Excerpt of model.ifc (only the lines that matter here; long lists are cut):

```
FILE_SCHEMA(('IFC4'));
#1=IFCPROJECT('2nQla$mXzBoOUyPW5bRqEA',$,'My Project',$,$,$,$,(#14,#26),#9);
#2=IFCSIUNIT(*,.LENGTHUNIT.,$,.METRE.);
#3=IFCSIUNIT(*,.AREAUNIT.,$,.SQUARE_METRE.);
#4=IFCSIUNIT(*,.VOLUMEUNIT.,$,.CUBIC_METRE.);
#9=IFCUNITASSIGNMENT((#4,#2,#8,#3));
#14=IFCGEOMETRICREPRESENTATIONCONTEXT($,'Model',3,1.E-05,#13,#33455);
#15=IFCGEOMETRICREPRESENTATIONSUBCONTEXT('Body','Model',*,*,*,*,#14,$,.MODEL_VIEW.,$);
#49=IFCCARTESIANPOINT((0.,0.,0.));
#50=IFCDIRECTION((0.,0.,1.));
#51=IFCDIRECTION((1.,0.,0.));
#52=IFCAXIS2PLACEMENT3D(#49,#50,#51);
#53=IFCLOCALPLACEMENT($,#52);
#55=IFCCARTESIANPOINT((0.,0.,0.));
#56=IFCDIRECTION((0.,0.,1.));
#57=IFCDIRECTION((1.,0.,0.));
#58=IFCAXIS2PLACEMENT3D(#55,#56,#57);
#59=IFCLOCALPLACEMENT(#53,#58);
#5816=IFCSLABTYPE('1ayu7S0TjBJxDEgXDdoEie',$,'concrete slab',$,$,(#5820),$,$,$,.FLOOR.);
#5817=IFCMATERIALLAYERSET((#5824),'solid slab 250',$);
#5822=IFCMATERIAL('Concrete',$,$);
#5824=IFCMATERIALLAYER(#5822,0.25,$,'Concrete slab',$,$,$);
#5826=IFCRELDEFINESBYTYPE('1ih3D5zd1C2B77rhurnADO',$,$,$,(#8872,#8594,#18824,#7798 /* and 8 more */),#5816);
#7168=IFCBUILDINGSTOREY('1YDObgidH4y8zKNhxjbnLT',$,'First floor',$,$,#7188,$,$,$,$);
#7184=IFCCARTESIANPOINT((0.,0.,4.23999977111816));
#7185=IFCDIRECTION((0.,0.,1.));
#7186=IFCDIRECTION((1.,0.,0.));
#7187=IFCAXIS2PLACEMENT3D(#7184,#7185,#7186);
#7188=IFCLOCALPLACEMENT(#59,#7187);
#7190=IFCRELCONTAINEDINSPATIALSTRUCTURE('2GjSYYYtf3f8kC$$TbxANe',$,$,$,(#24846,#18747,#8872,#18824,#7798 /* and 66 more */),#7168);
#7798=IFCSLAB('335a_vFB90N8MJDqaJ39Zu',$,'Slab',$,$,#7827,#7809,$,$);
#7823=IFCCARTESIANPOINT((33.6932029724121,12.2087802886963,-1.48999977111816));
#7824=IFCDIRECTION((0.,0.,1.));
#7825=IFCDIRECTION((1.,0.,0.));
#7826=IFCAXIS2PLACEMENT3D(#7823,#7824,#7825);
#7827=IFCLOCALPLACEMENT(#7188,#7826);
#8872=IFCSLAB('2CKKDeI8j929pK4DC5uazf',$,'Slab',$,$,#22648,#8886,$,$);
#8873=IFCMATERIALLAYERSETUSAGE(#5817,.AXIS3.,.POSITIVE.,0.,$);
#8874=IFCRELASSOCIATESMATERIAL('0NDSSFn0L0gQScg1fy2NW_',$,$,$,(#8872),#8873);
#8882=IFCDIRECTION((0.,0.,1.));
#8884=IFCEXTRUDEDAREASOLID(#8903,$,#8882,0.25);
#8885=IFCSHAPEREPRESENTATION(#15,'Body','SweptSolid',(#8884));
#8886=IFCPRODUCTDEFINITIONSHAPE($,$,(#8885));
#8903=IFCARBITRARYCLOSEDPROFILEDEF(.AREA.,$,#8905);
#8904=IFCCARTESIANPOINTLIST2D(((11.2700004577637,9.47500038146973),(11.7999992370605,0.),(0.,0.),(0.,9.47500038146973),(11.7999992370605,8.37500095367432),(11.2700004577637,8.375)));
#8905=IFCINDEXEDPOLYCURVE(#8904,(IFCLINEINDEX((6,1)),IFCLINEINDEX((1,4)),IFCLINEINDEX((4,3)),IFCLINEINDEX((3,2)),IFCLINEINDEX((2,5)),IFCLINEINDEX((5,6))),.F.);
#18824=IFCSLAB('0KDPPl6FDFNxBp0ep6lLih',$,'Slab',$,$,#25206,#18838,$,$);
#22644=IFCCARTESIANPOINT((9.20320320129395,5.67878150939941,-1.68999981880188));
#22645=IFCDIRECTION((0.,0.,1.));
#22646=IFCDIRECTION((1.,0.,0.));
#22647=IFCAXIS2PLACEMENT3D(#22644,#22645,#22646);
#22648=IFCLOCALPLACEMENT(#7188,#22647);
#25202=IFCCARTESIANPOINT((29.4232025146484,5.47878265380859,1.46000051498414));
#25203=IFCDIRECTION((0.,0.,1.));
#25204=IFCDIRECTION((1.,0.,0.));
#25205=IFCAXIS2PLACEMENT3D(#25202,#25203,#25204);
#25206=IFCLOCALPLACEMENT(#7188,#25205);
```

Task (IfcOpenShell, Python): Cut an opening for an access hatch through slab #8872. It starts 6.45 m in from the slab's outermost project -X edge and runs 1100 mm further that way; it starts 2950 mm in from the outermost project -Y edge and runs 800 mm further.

```python
import numpy as np
import ifcopenshell
import ifcopenshell.api.feature
import ifcopenshell.api.geometry
import ifcopenshell.api.root
import ifcopenshell.geom
import ifcopenshell.util.placement
import ifcopenshell.util.representation
import ifcopenshell.util.shape
import ifcopenshell.util.unit

model = ifcopenshell.open("model.ifc")
unit_scale = ifcopenshell.util.unit.calculate_unit_scale(model)
settings = ifcopenshell.geom.settings()


def volume(element):
    """Net volume in cubic metres, openings subtracted."""
    shape = ifcopenshell.geom.create_shape(settings, element)
    return ifcopenshell.util.shape.get_volume(shape.geometry)


slab = model.by_id(8872)
before = volume(slab)

# Extent in the slab's own axes, in metres. The edges named are its -X and -Y sides.
slab_shape = ifcopenshell.geom.create_shape(settings, slab)
vertices = ifcopenshell.util.shape.get_vertices(slab_shape.geometry)
x_min, y_min, bottom = vertices.min(axis=0)
top = vertices[:, 2].max()

opening = ifcopenshell.api.root.create_entity(model, ifc_class="IfcOpeningElement", name="Access hatch opening", predefined_type="OPENING")
context = ifcopenshell.util.representation.get_context(model, "Model", "Body", "MODEL_VIEW")
width, depth = 1.1, 0.8
outline = [(0.0, 0.0), (width, 0.0), (width, depth), (0.0, depth), (0.0, 0.0)]
# Overshoot both faces by 50 mm so the cut is clean.
shape = ifcopenshell.api.geometry.add_slab_representation(
    model, context=context, depth=top - bottom + 0.1, polyline=outline
)
ifcopenshell.api.geometry.assign_representation(model, product=opening, representation=shape)

matrix = ifcopenshell.util.placement.get_local_placement(slab.ObjectPlacement)
matrix[:, 3] = matrix @ np.append(np.array([x_min + 6.45, y_min + 2.95, bottom - 0.05]) / unit_scale, 1.0)
ifcopenshell.api.geometry.edit_object_placement(model, product=opening, matrix=matrix, is_si=False)
ifcopenshell.api.feature.add_feature(model, feature=opening, element=slab)

after = volume(slab)

print(f"slab volume {before:.3f} -> {after:.3f} m3")

model.write("model_updated.ifc")
```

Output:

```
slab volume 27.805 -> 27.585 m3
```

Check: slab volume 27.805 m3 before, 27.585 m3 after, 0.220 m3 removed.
